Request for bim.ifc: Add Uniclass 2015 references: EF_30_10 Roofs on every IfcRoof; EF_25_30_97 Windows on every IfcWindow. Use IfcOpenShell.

First a look at what the model holds.

```python
import ifcopenshell

model = ifcopenshell.open("bim.ifc")
print(model.schema)
print("classifications:", [c.Name for c in model.by_type("IfcClassification")])
for ifc_class in ("IfcDoor", "IfcRoof", "IfcStair", "IfcWall", "IfcWindow"):
    print(ifc_class, len(model.by_type(ifc_class)))
```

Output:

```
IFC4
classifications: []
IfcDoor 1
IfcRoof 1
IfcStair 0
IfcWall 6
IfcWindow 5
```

```python
import ifcopenshell
import ifcopenshell.api.classification

model = ifcopenshell.open("bim.ifc")

system = ifcopenshell.api.classification.add_classification(model, classification="Uniclass 2015")

codes = {
    "IfcRoof": ("EF_30_10", "Roofs"),
    "IfcWindow": ("EF_25_30_97", "Windows"),
}
for ifc_class, (code, name) in codes.items():
    products = model.by_type(ifc_class)
    ifcopenshell.api.classification.add_reference(
        model, products=products, classification=system, identification=code, name=name
    )
    print(code, len(products))

model.write("bim_rev.ifc")
```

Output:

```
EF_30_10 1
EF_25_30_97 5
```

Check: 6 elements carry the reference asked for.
